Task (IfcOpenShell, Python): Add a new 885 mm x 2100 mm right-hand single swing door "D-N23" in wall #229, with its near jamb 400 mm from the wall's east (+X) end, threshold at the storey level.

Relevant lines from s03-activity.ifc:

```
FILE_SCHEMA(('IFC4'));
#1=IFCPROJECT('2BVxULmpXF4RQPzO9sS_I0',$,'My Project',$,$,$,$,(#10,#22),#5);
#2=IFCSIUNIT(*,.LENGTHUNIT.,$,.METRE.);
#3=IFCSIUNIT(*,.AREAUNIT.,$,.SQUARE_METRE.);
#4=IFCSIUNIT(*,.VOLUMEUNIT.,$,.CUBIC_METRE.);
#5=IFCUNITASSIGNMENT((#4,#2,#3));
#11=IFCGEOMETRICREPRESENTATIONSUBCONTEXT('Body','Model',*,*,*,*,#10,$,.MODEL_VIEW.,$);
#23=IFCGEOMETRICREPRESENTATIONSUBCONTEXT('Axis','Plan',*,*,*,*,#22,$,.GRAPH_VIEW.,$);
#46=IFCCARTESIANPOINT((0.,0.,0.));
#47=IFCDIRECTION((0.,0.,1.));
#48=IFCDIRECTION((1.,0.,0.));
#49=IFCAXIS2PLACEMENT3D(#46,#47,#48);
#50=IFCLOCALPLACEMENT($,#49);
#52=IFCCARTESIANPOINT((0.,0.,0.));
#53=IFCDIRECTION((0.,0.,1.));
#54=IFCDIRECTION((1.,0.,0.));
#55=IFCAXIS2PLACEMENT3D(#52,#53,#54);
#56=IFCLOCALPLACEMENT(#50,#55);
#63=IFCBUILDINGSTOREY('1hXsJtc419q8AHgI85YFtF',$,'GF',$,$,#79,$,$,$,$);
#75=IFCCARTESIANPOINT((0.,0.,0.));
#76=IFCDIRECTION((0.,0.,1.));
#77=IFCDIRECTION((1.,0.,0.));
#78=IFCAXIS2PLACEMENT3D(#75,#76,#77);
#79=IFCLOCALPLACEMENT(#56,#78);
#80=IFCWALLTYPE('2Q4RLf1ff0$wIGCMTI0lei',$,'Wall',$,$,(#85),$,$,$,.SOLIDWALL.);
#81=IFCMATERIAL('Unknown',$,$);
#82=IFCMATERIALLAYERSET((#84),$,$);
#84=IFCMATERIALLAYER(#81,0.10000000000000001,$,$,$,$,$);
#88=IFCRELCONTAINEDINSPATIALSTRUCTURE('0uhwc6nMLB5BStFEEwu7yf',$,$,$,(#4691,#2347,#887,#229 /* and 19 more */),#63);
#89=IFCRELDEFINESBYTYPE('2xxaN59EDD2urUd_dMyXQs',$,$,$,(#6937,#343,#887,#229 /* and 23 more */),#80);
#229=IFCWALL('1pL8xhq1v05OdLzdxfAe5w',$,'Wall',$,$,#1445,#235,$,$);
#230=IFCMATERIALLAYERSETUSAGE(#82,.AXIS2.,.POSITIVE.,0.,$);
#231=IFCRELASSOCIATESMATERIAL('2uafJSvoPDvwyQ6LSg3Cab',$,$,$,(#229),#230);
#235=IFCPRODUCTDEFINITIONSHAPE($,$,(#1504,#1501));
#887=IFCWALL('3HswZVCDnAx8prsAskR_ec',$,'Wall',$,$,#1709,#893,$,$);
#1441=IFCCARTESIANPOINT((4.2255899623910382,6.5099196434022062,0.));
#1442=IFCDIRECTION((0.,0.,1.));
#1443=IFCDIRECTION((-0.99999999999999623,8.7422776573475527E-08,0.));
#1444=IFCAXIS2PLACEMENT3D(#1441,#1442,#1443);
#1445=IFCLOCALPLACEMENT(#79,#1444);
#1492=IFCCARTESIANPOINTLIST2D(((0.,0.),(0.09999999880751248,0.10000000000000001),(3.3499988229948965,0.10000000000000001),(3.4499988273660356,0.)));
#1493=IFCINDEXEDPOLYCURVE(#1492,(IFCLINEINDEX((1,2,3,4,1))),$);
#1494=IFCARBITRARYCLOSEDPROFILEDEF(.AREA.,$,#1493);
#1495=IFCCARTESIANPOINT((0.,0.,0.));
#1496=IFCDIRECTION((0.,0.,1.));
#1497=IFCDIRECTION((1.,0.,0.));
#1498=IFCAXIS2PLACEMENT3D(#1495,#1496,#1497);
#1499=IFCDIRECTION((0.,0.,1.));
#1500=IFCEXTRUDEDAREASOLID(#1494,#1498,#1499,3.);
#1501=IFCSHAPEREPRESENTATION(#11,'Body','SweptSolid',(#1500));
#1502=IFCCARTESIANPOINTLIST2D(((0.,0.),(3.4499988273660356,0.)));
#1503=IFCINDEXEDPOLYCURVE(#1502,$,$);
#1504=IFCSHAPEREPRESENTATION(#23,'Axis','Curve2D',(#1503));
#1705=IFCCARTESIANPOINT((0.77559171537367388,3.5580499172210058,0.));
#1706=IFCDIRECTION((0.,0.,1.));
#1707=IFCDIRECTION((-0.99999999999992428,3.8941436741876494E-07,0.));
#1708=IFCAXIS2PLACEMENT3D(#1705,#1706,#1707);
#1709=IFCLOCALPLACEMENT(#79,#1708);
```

```python
import numpy as np
import ifcopenshell
import ifcopenshell.api.feature
import ifcopenshell.api.geometry
import ifcopenshell.api.root
import ifcopenshell.api.spatial
import ifcopenshell.geom
import ifcopenshell.util.element
import ifcopenshell.util.placement
import ifcopenshell.util.representation
import ifcopenshell.util.shape
import ifcopenshell.util.unit

model = ifcopenshell.open("s03-activity.ifc")
unit_scale = ifcopenshell.util.unit.calculate_unit_scale(model)
settings = ifcopenshell.geom.settings()


def volume(element):
    """Net volume in cubic metres, openings subtracted."""
    shape = ifcopenshell.geom.create_shape(settings, element)
    return ifcopenshell.util.shape.get_volume(shape.geometry)


wall = model.by_guid("1pL8xhq1v05OdLzdxfAe5w")
storey = ifcopenshell.util.element.get_container(wall, ifc_class="IfcBuildingStorey")
context = ifcopenshell.util.representation.get_context(model, "Model", "Body", "MODEL_VIEW")
before = volume(wall)

width, height, from_end, sill = 0.885, 2.1, 0.4, 0.0  # metres

# The wall runs along its own X axis, and the end named is its -X end.
wall_shape = ifcopenshell.geom.create_shape(settings, wall)
x, y, z = ifcopenshell.util.shape.get_vertices(wall_shape.geometry).T
start = x.min() + from_end
face, thickness = float(y.min()), float(y.max() - y.min())
wall_matrix = ifcopenshell.util.placement.get_local_placement(wall.ObjectPlacement)
level = ifcopenshell.util.placement.get_local_placement(storey.ObjectPlacement)[2, 3]


def in_wall(x, y):
    """Placement at x, y metres in the wall's axes, at sill height."""
    matrix = wall_matrix.copy()
    matrix[:, 3] = wall_matrix @ np.array([x / unit_scale, y / unit_scale, 0.0, 1.0])
    matrix[2, 3] = level + sill / unit_scale
    return matrix


# Opening: a box that overshoots both wall faces by 50 mm.
opening = ifcopenshell.api.root.create_entity(model, ifc_class="IfcOpeningElement", predefined_type="OPENING")
box = ifcopenshell.api.geometry.add_wall_representation(
    model, context=context, length=width, height=height, thickness=thickness + 0.1
)
ifcopenshell.api.geometry.assign_representation(model, product=opening, representation=box)
ifcopenshell.api.geometry.edit_object_placement(model, product=opening, matrix=in_wall(start, face - 0.05), is_si=False)
ifcopenshell.api.feature.add_feature(model, feature=opening, element=wall)

door = ifcopenshell.api.root.create_entity(model, ifc_class="IfcDoor", name="D-N23", predefined_type="DOOR")
door.OverallWidth, door.OverallHeight = width / unit_scale, height / unit_scale
door.OperationType = "SINGLE_SWING_RIGHT"
body = ifcopenshell.api.geometry.add_door_representation(
    model,
    context=context,
    overall_width=door.OverallWidth,
    overall_height=door.OverallHeight,
    operation_type="SINGLE_SWING_RIGHT",
    lining_properties={"LiningDepth": thickness / unit_scale, "ThresholdDepth": thickness / unit_scale},
)
ifcopenshell.api.geometry.assign_representation(model, product=door, representation=body)
ifcopenshell.api.spatial.assign_container(model, products=[door], relating_structure=storey)
ifcopenshell.api.feature.add_filling(model, opening=opening, element=door)

# The lining spans the wall, so the door starts at the wall face.
ifcopenshell.api.geometry.edit_object_placement(model, product=door, matrix=in_wall(start, face), is_si=False)

after = volume(wall)

print(f"wall volume {before:.3f} -> {after:.3f} m3")

model.write("s03-activity_rev.ifc")
```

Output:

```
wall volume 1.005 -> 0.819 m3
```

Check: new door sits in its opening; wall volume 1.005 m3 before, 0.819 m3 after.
